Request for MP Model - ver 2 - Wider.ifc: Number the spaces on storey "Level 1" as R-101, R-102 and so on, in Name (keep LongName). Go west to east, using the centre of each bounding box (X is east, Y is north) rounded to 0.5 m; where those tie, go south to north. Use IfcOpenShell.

First a look at what the model holds.

```python
import ifcopenshell
import ifcopenshell.util.element
import ifcopenshell.util.placement

model = ifcopenshell.open("MP Model - ver 2 - Wider.ifc")
print(model.schema)
storey = next(s for s in model.by_type("IfcBuildingStorey") if s.Name == "Level 1")
spaces = [e for e in ifcopenshell.util.element.get_decomposition(storey) if e.is_a("IfcSpace")]
for e in sorted(spaces, key=lambda e: e.id()):
    origin = ifcopenshell.util.placement.get_local_placement(e.ObjectPlacement)[:3, 3]
    print(e.id(), e.Name, e.LongName, origin.round(2) + 0.0, sep=" | ")
```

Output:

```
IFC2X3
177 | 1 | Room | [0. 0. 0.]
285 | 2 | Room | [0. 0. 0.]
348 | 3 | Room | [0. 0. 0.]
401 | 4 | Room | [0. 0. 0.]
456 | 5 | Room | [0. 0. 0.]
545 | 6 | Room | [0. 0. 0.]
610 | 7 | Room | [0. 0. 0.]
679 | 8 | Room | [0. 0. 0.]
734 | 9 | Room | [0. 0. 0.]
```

```python
import ifcopenshell
import ifcopenshell.geom
import ifcopenshell.util.element
import ifcopenshell.util.shape

model = ifcopenshell.open("MP Model - ver 2 - Wider.ifc")
settings = ifcopenshell.geom.settings()
settings.set("use-world-coords", True)


def centre(element):
    shape = ifcopenshell.geom.create_shape(settings, element)
    return ifcopenshell.util.shape.get_bbox_centroid(shape.geometry)


storey = next(s for s in model.by_type("IfcBuildingStorey") if s.Name == "Level 1")
spaces = [e for e in ifcopenshell.util.element.get_decomposition(storey) if e.is_a("IfcSpace")]

# Insertion points can sit at a corner or the storey origin, so sort by the geometry (in metres).
centres = {e: centre(e) for e in spaces}
spaces.sort(key=lambda e: (round(centres[e][0] / 0.5), centres[e][1]))

for i, e in enumerate(spaces, start=1):
    number = f"R-1{i:02d}"
    e.Name = number
    print(e.id(), number)

model.write("MP Model - ver 2 - Wider_v2.ifc")
```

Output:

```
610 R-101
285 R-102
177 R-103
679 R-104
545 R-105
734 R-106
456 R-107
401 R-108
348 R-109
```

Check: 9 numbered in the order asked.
